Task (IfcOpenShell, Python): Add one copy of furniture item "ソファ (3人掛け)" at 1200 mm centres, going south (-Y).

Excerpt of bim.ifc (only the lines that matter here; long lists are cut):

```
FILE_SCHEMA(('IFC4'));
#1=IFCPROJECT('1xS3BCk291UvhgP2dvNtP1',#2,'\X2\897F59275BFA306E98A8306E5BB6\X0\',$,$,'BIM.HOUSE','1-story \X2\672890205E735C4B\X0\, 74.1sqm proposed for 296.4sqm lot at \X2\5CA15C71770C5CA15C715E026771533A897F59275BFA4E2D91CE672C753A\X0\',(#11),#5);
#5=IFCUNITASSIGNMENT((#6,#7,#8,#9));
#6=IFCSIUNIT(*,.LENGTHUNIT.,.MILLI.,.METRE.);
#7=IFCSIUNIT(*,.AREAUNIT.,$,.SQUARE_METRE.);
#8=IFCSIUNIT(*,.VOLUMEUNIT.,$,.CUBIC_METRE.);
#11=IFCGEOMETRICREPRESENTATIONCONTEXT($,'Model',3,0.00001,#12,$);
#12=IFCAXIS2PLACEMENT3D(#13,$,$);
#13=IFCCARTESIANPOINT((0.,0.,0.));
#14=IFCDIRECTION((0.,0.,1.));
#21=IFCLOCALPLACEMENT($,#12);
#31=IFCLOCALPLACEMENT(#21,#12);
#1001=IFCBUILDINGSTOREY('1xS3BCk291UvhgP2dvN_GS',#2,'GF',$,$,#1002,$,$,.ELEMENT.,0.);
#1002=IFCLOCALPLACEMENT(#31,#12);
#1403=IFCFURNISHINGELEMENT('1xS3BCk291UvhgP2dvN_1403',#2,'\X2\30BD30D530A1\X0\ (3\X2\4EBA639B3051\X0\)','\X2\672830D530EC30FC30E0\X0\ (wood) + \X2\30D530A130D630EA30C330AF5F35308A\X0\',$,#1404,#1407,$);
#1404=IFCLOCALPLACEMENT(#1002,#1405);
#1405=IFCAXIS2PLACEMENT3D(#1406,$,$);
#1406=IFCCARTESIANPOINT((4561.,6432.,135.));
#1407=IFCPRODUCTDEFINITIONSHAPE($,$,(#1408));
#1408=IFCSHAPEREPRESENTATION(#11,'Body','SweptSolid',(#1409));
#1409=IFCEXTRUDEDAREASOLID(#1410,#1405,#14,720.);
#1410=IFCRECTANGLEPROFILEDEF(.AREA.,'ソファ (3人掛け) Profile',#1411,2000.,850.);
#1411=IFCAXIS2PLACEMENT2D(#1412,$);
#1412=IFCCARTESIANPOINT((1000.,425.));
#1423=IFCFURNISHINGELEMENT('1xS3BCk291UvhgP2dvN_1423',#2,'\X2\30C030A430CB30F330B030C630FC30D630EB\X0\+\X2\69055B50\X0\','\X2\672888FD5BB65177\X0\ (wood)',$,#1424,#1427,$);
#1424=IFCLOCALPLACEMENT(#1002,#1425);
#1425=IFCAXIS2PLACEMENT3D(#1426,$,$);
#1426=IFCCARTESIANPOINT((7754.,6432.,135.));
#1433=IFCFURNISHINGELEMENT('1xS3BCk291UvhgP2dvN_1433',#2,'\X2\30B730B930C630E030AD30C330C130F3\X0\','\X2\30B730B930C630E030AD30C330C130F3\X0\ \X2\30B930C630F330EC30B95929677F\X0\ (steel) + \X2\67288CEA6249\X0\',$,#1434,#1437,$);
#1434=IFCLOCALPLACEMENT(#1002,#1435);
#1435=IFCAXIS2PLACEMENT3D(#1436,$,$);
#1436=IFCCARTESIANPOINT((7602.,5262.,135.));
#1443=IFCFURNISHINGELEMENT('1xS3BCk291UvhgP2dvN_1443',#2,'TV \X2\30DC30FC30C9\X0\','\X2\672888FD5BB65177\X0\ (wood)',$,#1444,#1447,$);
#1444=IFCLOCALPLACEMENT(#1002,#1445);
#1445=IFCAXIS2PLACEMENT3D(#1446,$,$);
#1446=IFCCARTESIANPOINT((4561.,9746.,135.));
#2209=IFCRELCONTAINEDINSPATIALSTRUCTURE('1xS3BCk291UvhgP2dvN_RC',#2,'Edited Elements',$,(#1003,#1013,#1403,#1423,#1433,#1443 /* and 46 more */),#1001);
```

```python
import numpy as np
import ifcopenshell
import ifcopenshell.api.geometry
import ifcopenshell.api.root
import ifcopenshell.util.element
import ifcopenshell.util.placement
import ifcopenshell.util.unit

model = ifcopenshell.open("bim.ifc")
unit_scale = ifcopenshell.util.unit.calculate_unit_scale(model)


def reuse_history(source, copy):
    """copy_class also copies each property set's owner history, people and application; keep the originals."""
    for rel in copy.IsDefinedBy:
        if rel.is_a("IfcRelDefinesByProperties") and (history := rel.RelatingPropertyDefinition.OwnerHistory):
            rel.RelatingPropertyDefinition.OwnerHistory = source.OwnerHistory
            ifcopenshell.util.element.remove_deep2(model, history)


source = model.by_guid("1xS3BCk291UvhgP2dvN_1403")
base = ifcopenshell.util.placement.get_local_placement(source.ObjectPlacement)
step = np.array([0.0, -1.0, 0.0]) * 1.2 / unit_scale

for i in range(1, 2):
    copy = ifcopenshell.api.root.copy_class(model, product=source)
    copy.Representation = ifcopenshell.util.element.copy_deep(
        model, source.Representation, exclude=["IfcGeometricRepresentationContext", "IfcRepresentationMap"]
    )
    reuse_history(source, copy)
    matrix = base.copy()
    matrix[:3, 3] += i * step
    print("added at", matrix[:3, 3].round(3) + 0.0)
    ifcopenshell.api.geometry.edit_object_placement(model, product=copy, matrix=matrix, is_si=False)

model.write("bim-out.ifc")
```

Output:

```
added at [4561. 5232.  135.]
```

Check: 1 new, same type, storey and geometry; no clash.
